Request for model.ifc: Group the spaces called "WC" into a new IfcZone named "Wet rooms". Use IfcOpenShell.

First a look at what the model holds.

```python
import ifcopenshell

model = ifcopenshell.open("model.ifc")
print(model.schema)
seen = {}
for space in model.by_type("IfcSpace"):
    seen[space.LongName] = seen.get(space.LongName, 0) + 1
for name, count in sorted(seen.items(), key=str):
    print(count, "x", name)
print("zones:", [z.Name for z in model.by_type("IfcZone")][:20])
```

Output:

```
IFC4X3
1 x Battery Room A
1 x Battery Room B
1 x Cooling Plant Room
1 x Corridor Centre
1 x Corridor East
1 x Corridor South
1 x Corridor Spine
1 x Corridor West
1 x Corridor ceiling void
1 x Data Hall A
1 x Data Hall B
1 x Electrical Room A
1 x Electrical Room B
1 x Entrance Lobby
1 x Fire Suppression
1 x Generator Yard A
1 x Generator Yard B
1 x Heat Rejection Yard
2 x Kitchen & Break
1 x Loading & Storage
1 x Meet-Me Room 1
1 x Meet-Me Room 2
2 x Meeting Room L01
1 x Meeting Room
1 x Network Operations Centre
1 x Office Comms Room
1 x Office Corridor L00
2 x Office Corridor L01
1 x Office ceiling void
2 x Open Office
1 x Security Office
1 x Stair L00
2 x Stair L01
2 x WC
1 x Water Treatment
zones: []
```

```python
import ifcopenshell
import ifcopenshell.api.group
import ifcopenshell.api.root

model = ifcopenshell.open("model.ifc")

names = {"WC"}
spaces = [s for s in model.by_type("IfcSpace") if s.LongName in names]

zone = ifcopenshell.api.root.create_entity(model, ifc_class="IfcZone", name="Wet rooms")
ifcopenshell.api.group.assign_group(model, products=spaces, group=zone)
print(len(spaces), "spaces in", zone.Name)

model.write("model_edited.ifc")
```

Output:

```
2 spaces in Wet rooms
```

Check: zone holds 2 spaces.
